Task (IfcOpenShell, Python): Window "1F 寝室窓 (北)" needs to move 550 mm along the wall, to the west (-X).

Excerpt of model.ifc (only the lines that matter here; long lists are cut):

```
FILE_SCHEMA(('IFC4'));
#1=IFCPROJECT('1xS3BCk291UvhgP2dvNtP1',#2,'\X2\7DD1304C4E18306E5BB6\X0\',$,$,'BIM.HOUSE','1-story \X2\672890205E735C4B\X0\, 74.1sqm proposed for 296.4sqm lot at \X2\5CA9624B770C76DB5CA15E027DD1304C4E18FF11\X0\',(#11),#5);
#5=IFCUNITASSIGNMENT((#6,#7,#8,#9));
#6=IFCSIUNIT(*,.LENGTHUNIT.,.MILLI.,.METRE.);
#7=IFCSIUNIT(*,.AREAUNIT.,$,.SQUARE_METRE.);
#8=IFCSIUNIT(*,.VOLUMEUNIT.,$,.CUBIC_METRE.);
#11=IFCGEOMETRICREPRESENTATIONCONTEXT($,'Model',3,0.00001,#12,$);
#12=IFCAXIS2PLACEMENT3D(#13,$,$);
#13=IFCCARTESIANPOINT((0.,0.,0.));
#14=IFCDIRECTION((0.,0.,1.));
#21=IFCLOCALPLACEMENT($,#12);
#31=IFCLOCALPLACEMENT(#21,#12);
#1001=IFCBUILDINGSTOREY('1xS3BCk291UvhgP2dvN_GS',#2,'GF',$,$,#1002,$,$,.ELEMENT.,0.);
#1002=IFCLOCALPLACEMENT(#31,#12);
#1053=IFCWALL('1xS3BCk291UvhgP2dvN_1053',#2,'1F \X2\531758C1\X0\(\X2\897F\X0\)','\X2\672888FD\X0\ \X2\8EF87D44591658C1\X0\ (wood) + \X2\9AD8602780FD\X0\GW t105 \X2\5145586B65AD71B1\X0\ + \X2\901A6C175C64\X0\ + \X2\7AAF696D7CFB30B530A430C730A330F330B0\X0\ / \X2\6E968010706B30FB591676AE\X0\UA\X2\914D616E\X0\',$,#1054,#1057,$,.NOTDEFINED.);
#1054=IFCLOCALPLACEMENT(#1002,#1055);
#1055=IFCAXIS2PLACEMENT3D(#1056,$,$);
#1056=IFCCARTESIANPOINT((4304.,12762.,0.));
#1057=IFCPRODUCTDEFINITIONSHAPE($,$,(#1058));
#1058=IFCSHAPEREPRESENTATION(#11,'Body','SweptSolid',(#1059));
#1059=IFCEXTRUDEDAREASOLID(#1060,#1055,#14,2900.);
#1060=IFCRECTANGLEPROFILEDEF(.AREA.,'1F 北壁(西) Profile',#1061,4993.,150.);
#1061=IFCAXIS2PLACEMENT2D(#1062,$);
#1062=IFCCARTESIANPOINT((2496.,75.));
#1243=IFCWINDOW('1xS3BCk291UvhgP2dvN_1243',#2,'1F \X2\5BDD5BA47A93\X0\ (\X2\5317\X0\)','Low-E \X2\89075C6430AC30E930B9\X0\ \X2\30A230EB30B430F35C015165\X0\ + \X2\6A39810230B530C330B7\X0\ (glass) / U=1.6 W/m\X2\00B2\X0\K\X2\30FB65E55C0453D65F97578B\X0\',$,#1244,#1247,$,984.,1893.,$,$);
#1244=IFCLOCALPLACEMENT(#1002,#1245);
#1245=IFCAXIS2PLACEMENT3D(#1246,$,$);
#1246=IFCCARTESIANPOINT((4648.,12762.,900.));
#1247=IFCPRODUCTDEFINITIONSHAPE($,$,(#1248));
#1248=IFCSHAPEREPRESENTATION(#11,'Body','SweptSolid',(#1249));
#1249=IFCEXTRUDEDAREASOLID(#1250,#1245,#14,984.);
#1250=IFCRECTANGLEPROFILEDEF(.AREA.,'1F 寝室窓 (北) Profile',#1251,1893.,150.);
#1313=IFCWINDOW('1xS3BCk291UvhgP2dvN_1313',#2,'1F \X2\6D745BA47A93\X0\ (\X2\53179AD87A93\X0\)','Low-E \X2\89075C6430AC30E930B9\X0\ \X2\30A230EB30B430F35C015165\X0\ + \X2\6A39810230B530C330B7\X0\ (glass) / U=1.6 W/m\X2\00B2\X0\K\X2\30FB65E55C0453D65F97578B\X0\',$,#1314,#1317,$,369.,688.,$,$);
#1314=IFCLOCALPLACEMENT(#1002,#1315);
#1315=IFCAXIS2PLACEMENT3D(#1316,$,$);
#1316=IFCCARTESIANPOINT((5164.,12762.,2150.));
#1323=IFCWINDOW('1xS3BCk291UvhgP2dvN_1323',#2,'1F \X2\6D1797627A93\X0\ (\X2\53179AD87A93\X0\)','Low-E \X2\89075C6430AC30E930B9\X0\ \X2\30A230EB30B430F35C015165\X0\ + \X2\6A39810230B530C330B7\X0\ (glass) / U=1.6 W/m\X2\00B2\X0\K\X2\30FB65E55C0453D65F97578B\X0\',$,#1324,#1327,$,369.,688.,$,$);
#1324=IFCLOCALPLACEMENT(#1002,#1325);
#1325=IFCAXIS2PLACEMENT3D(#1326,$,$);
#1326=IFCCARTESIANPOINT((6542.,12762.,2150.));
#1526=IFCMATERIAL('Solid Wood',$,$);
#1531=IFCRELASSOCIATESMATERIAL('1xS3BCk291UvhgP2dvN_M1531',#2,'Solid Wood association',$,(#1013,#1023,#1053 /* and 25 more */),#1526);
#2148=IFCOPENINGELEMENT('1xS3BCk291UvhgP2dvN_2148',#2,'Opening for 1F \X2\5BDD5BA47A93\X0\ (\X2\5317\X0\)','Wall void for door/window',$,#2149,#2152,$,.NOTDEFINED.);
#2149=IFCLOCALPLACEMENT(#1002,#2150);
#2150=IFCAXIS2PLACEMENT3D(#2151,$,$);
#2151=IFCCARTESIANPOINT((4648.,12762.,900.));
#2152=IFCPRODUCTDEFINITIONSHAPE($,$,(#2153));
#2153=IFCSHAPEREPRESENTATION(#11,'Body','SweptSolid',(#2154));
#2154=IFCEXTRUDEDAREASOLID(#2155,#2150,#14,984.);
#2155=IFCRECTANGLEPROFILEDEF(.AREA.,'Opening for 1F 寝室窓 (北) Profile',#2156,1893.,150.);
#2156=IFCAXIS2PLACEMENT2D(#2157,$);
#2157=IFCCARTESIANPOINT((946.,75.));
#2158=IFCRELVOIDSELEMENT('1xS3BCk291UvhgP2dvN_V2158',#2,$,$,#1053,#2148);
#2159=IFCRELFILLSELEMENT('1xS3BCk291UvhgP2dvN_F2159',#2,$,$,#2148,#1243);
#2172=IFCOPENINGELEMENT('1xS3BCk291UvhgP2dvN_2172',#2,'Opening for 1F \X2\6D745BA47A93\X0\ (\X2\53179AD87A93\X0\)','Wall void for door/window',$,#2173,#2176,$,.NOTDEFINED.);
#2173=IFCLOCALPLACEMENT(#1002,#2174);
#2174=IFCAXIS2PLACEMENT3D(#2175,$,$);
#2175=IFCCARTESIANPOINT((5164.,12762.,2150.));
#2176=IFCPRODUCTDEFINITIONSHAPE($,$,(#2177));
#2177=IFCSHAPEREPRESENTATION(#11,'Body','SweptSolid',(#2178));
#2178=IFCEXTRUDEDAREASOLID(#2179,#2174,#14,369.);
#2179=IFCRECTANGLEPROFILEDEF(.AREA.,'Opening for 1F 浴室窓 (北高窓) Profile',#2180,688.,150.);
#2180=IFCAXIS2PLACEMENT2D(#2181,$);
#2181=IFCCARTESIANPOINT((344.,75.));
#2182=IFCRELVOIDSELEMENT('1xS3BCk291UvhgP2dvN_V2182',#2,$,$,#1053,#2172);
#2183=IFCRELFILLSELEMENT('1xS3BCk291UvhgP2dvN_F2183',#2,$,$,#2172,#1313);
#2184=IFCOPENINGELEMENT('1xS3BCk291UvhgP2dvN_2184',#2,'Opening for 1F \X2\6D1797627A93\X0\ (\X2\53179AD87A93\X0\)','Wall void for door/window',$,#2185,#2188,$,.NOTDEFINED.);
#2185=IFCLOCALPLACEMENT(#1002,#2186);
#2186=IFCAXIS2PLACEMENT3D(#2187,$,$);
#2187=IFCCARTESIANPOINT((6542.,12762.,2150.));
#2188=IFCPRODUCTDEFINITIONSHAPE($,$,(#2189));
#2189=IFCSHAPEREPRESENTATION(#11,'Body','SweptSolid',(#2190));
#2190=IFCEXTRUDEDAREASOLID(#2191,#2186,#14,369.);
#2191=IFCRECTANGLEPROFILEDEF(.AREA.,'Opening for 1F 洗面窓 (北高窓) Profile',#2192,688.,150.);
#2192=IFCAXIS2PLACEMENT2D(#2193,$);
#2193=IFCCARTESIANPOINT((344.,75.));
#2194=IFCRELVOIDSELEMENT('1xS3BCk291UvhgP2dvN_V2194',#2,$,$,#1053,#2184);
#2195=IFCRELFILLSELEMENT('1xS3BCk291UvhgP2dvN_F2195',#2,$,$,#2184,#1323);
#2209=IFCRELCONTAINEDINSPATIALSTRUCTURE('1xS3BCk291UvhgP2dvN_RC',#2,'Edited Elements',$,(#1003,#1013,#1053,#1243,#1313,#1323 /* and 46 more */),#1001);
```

```python
import ifcopenshell
import ifcopenshell.api.geometry
import ifcopenshell.util.placement
import ifcopenshell.util.unit

model = ifcopenshell.open("model.ifc")
unit_scale = ifcopenshell.util.unit.calculate_unit_scale(model)

window = model.by_guid("1xS3BCk291UvhgP2dvN_1243")
opening = window.FillsVoids[0].RelatingOpeningElement
wall = opening.VoidsElements[0].RelatingBuildingElement

wall_matrix = ifcopenshell.util.placement.get_local_placement(wall.ObjectPlacement)
shift = wall_matrix[:3, 0] * -0.55 / unit_scale
before = ifcopenshell.util.placement.get_local_placement(window.ObjectPlacement)[:3, 3].copy()

# The window is not placed relative to its opening, so move both.
for product in (opening, window):
    matrix = ifcopenshell.util.placement.get_local_placement(product.ObjectPlacement)
    matrix[:3, 3] += shift
    ifcopenshell.api.geometry.edit_object_placement(model, product=product, matrix=matrix, is_si=False)

after = ifcopenshell.util.placement.get_local_placement(window.ObjectPlacement)[:3, 3]
print("window moved by", (after - before).round(3) + 0.0)

model.write("model-out.ifc")
```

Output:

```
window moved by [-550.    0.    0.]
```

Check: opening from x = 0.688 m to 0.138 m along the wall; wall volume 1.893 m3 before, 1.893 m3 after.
